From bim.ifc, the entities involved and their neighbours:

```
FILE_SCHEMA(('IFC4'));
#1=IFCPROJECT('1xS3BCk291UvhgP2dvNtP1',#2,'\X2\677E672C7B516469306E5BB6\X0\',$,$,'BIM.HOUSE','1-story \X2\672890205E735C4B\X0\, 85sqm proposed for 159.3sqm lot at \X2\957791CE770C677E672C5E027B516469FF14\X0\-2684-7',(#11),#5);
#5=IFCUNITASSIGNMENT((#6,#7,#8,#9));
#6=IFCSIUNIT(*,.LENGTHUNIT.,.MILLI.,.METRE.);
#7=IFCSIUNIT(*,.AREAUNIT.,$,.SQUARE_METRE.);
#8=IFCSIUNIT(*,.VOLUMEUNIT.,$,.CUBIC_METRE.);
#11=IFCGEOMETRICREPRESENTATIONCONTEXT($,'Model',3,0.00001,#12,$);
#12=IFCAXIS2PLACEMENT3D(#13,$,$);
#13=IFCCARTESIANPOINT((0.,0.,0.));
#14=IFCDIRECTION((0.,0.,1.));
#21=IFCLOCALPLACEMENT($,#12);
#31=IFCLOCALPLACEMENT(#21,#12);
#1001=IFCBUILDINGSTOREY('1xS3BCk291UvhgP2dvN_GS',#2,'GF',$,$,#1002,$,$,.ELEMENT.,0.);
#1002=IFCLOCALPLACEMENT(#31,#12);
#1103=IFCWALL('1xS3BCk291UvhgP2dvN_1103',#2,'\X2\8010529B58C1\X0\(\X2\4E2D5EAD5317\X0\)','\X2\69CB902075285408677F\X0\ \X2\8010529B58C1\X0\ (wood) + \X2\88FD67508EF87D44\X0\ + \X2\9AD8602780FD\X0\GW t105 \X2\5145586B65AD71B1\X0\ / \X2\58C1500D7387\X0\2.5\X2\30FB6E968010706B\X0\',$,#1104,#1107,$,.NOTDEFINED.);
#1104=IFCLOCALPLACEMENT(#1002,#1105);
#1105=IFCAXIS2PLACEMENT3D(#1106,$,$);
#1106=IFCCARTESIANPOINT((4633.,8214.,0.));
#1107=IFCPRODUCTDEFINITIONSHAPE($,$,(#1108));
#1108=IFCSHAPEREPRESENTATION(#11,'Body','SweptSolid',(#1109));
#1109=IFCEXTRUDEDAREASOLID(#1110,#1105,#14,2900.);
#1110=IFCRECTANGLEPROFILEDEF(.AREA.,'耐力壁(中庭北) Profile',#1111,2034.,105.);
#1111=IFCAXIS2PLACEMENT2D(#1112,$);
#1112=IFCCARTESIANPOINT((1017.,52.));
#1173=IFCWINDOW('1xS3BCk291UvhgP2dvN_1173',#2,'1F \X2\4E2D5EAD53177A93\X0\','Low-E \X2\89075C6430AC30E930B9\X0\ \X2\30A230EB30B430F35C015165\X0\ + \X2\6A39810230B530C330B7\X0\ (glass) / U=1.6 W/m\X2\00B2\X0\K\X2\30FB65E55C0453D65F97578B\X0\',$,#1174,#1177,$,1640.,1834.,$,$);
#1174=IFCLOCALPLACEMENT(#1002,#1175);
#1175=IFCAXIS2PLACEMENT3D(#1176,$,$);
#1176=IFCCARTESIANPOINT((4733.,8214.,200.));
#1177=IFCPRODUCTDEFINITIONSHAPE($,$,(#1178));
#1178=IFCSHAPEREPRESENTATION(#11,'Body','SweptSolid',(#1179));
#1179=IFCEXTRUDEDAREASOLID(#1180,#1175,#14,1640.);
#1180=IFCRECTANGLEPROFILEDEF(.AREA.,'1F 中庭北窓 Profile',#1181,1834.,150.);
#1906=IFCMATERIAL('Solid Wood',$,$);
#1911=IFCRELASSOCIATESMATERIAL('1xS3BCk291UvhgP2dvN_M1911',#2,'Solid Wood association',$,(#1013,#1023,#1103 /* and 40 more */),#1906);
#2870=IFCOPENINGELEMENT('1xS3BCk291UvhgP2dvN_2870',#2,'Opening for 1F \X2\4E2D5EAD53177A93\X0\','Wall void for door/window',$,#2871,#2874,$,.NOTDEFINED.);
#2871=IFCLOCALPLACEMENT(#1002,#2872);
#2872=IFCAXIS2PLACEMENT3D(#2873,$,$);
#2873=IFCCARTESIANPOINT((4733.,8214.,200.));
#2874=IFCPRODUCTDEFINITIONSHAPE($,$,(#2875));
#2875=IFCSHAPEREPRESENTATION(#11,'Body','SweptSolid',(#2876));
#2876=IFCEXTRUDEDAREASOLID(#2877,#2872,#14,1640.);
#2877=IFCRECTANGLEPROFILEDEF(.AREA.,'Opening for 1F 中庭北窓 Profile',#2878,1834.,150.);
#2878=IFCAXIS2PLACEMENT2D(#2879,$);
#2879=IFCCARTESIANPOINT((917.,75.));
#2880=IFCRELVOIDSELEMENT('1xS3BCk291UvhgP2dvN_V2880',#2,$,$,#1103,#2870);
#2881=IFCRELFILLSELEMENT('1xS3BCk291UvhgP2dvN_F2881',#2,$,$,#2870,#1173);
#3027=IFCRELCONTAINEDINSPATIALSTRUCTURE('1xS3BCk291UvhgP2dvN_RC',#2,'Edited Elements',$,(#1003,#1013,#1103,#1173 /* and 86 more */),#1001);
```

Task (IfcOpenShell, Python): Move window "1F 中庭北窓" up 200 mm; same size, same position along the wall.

```python
import numpy as np
import ifcopenshell
import ifcopenshell.api.geometry
import ifcopenshell.util.placement
import ifcopenshell.util.unit

model = ifcopenshell.open("bim.ifc")
unit_scale = ifcopenshell.util.unit.calculate_unit_scale(model)

window = model.by_id(1173)
opening = window.FillsVoids[0].RelatingOpeningElement
dz = 0.2 / unit_scale

shift = np.array([0.0, 0.0, dz])
# The window is not placed relative to its opening, so move both.
for product in (opening, window):
    matrix = ifcopenshell.util.placement.get_local_placement(product.ObjectPlacement)
    matrix[:3, 3] += shift
    ifcopenshell.api.geometry.edit_object_placement(model, product=product, matrix=matrix, is_si=False)

print(f"moved by {dz * unit_scale:+.3f} m")

model.write("bim_v2.ifc")
```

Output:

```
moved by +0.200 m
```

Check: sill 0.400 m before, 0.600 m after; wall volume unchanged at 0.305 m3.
